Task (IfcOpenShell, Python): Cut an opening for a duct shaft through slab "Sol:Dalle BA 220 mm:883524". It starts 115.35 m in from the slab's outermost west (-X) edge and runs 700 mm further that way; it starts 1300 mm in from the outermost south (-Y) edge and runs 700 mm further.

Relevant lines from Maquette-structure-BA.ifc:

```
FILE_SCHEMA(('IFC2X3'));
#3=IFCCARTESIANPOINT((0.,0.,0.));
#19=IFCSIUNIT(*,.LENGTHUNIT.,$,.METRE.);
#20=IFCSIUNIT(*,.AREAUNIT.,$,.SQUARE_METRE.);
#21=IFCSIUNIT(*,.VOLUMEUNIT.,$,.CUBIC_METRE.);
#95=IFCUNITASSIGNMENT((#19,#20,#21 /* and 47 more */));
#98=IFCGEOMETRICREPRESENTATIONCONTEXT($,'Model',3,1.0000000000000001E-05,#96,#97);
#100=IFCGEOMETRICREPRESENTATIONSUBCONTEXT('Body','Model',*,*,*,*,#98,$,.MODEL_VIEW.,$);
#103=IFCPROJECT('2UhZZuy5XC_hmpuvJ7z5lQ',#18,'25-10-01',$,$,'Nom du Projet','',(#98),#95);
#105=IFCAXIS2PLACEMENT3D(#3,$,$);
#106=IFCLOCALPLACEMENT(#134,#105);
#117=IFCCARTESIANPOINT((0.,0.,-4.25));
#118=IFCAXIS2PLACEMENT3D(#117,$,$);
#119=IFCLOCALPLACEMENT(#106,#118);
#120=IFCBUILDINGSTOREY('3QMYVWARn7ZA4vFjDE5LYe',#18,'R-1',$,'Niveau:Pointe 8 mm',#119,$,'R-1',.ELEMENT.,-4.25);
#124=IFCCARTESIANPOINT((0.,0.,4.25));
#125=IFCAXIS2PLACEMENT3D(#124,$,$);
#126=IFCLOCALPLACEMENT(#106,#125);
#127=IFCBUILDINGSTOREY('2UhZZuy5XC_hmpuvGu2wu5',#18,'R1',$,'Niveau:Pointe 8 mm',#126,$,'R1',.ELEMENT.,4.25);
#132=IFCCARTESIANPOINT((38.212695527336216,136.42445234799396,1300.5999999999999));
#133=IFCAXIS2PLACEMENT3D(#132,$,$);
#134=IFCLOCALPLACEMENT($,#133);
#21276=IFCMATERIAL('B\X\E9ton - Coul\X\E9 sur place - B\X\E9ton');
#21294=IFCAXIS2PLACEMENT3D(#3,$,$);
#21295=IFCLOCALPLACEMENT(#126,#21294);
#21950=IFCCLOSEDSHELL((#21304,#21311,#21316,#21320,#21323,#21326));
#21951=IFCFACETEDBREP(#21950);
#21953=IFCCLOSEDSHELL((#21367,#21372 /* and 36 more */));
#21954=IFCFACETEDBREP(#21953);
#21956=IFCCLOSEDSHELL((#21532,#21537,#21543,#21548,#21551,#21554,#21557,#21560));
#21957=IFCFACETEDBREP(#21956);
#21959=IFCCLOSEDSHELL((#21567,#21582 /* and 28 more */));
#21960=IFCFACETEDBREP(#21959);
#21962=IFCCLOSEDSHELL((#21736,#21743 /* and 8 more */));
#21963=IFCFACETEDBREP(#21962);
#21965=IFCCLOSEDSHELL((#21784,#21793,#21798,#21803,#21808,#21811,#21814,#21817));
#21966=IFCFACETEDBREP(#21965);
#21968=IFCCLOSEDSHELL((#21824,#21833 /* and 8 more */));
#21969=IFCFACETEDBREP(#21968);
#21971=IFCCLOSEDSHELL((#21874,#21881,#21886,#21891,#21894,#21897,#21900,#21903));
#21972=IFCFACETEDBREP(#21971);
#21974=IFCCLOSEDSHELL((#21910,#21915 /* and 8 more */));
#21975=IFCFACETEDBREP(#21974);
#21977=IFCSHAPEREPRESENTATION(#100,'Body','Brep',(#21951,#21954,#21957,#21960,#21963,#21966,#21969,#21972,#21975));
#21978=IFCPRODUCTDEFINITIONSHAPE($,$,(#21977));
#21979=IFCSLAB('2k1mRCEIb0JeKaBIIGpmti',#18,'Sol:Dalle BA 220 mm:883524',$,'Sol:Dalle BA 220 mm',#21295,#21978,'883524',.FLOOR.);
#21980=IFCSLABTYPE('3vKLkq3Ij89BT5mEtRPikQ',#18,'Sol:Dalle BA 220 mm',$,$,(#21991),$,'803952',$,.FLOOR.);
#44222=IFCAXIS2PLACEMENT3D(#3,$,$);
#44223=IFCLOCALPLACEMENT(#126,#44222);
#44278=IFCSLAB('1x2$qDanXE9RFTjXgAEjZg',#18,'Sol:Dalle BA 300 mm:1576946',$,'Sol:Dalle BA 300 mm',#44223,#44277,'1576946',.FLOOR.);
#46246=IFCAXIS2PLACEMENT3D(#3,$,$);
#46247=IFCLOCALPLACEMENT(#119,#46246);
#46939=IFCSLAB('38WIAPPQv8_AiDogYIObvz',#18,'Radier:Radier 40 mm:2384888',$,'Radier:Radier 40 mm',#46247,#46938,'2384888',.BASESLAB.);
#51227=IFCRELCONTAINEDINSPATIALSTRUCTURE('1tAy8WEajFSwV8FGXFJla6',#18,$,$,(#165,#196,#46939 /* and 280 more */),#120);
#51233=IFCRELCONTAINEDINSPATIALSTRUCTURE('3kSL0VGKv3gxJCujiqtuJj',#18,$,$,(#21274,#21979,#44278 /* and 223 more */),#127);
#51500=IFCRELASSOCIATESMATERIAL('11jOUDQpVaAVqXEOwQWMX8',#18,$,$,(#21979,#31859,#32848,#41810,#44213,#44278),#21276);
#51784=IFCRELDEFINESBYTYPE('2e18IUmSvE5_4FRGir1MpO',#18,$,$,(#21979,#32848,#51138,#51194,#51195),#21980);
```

```python
import numpy as np
import ifcopenshell
import ifcopenshell.api.feature
import ifcopenshell.api.geometry
import ifcopenshell.api.root
import ifcopenshell.geom
import ifcopenshell.util.placement
import ifcopenshell.util.representation
import ifcopenshell.util.shape
import ifcopenshell.util.unit

model = ifcopenshell.open("Maquette-structure-BA.ifc")
unit_scale = ifcopenshell.util.unit.calculate_unit_scale(model)
settings = ifcopenshell.geom.settings()


def volume(element):
    """Net volume in cubic metres, openings subtracted."""
    shape = ifcopenshell.geom.create_shape(settings, element)
    return ifcopenshell.util.shape.get_volume(shape.geometry)


slab = model.by_guid("2k1mRCEIb0JeKaBIIGpmti")
before = volume(slab)

# Extent in the slab's own axes, in metres. The edges named are its -X and -Y sides.
slab_shape = ifcopenshell.geom.create_shape(settings, slab)
vertices = ifcopenshell.util.shape.get_vertices(slab_shape.geometry)
x_min, y_min, bottom = vertices.min(axis=0)
top = vertices[:, 2].max()

opening = ifcopenshell.api.root.create_entity(model, ifc_class="IfcOpeningElement", name="Duct shaft opening")
context = ifcopenshell.util.representation.get_context(model, "Model", "Body", "MODEL_VIEW")
width, depth = 0.7, 0.7
outline = [(0.0, 0.0), (width, 0.0), (width, depth), (0.0, depth), (0.0, 0.0)]
# Overshoot both faces by 50 mm so the cut is clean.
shape = ifcopenshell.api.geometry.add_slab_representation(
    model, context=context, depth=top - bottom + 0.1, polyline=outline
)
ifcopenshell.api.geometry.assign_representation(model, product=opening, representation=shape)

matrix = ifcopenshell.util.placement.get_local_placement(slab.ObjectPlacement)
matrix[:, 3] = matrix @ np.append(np.array([x_min + 115.35, y_min + 1.3, bottom - 0.05]) / unit_scale, 1.0)
ifcopenshell.api.geometry.edit_object_placement(model, product=opening, matrix=matrix, is_si=False)
ifcopenshell.api.feature.add_feature(model, feature=opening, element=slab)

after = volume(slab)

print(f"slab volume {before:.3f} -> {after:.3f} m3")

model.write("Maquette-structure-BA_updated.ifc")
```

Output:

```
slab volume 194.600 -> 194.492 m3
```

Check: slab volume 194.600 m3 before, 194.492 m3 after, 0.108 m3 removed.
